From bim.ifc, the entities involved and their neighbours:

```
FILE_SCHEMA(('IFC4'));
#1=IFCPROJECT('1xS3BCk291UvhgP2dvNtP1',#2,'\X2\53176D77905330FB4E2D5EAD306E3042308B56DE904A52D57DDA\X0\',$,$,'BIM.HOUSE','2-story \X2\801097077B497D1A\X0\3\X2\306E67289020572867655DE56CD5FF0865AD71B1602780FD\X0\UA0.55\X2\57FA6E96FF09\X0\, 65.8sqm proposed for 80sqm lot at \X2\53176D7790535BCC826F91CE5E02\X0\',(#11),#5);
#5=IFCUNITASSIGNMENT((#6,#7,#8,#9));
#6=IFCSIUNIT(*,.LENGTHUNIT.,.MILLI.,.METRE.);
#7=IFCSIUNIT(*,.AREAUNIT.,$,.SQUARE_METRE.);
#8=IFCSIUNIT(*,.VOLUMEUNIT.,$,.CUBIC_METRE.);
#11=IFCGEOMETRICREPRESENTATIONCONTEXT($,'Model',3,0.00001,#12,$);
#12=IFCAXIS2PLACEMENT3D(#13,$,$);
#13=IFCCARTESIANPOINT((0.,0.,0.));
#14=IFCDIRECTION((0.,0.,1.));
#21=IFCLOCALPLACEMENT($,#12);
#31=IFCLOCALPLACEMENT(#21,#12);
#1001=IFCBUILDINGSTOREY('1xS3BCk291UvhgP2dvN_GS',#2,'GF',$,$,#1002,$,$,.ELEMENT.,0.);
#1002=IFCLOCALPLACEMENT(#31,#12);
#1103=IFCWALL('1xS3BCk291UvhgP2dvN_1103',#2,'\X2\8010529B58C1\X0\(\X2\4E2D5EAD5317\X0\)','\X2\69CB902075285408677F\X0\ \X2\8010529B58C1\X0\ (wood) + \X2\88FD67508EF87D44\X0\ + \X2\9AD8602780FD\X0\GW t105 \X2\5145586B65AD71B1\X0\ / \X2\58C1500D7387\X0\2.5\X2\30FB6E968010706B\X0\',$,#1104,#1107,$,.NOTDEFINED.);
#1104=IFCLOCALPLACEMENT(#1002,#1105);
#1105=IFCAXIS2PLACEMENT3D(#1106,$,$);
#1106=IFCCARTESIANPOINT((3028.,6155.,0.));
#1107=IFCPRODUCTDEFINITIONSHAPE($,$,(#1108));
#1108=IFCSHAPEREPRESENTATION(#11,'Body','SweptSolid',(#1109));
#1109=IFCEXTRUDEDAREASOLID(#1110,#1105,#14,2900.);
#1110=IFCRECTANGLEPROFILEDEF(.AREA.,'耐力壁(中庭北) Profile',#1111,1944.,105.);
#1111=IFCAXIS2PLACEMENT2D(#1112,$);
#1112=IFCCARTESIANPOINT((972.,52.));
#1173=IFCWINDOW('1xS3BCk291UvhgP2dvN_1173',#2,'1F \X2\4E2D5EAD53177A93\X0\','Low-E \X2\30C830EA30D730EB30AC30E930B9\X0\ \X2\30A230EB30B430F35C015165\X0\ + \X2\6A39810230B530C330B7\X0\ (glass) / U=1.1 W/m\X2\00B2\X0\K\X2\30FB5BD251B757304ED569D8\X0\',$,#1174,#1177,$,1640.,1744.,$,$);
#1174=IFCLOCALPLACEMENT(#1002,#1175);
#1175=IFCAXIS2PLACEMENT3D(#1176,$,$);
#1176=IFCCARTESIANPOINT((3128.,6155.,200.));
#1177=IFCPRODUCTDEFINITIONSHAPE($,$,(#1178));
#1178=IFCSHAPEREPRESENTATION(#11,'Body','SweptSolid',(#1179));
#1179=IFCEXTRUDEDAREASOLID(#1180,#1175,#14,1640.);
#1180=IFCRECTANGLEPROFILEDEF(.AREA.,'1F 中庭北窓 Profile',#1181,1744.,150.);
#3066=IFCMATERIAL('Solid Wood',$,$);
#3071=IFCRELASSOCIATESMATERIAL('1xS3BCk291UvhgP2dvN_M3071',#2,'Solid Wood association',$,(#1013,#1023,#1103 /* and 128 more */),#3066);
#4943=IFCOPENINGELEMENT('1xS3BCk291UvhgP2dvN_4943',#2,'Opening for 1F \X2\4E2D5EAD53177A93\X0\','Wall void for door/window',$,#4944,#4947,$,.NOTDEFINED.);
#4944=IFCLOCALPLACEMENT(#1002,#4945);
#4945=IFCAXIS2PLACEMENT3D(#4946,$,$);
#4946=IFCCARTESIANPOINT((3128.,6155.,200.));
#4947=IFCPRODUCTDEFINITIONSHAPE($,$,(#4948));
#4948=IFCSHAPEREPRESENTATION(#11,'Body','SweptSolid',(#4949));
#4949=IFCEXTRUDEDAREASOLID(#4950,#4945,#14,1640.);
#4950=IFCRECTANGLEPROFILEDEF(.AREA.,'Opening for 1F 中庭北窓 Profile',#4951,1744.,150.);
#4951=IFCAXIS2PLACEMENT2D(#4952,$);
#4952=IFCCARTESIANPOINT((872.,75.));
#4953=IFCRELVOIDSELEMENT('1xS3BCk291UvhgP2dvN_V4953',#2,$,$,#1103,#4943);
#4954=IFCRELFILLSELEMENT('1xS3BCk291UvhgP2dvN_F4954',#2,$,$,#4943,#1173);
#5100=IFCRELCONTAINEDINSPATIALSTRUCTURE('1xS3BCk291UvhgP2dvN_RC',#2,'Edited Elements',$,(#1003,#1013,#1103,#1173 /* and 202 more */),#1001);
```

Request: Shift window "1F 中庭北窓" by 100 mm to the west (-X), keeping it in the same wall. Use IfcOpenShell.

```python
import ifcopenshell
import ifcopenshell.api.geometry
import ifcopenshell.util.placement
import ifcopenshell.util.unit

model = ifcopenshell.open("bim.ifc")
unit_scale = ifcopenshell.util.unit.calculate_unit_scale(model)

window = model.by_id(1173)
opening = window.FillsVoids[0].RelatingOpeningElement
wall = opening.VoidsElements[0].RelatingBuildingElement

wall_matrix = ifcopenshell.util.placement.get_local_placement(wall.ObjectPlacement)
shift = wall_matrix[:3, 0] * -0.1 / unit_scale
before = ifcopenshell.util.placement.get_local_placement(window.ObjectPlacement)[:3, 3].copy()

# The window is not placed relative to its opening, so move both.
for product in (opening, window):
    matrix = ifcopenshell.util.placement.get_local_placement(product.ObjectPlacement)
    matrix[:3, 3] += shift
    ifcopenshell.api.geometry.edit_object_placement(model, product=product, matrix=matrix, is_si=False)

after = ifcopenshell.util.placement.get_local_placement(window.ObjectPlacement)[:3, 3]
print("window moved by", (after - before).round(3) + 0.0)

model.write("bim_v2.ifc")
```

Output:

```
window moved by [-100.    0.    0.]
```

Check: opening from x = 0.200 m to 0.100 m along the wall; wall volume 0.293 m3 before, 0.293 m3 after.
